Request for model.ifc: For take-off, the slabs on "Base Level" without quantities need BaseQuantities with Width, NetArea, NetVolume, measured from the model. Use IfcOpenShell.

First a look at what the model holds.

```python
import ifcopenshell
import ifcopenshell.util.element
import ifcopenshell.util.unit

model = ifcopenshell.open("model.ifc")
print(model.schema)
for unit_type in ("LENGTHUNIT", "AREAUNIT", "VOLUMEUNIT"):
    print(unit_type, ifcopenshell.util.unit.calculate_unit_scale(model, unit_type))
storey = next(s for s in model.by_type("IfcBuildingStorey") if s.Name == "Base Level")
slabs = [e for e in ifcopenshell.util.element.get_decomposition(storey) if e.is_a("IfcSlab")]
for e in sorted(slabs, key=lambda e: e.id()):
    print(e.id(), e.is_a(), e.Name, list(ifcopenshell.util.element.get_psets(e, qtos_only=True)), sep=" | ")
```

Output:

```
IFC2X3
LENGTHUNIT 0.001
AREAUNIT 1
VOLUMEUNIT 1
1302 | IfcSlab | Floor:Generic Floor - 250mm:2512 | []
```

```python
import ifcopenshell
import ifcopenshell.api.pset
import ifcopenshell.geom
import ifcopenshell.util.element
import ifcopenshell.util.shape
import ifcopenshell.util.unit

model = ifcopenshell.open("model.ifc")
unit_scale = ifcopenshell.util.unit.calculate_unit_scale(model)
area_scale = ifcopenshell.util.unit.calculate_unit_scale(model, "AREAUNIT")
volume_scale = ifcopenshell.util.unit.calculate_unit_scale(model, "VOLUMEUNIT")
settings = ifcopenshell.geom.settings()

storey = next(s for s in model.by_type("IfcBuildingStorey") if s.Name == "Base Level")
slabs = [e for e in ifcopenshell.util.element.get_decomposition(storey) if e.is_a("IfcSlab")]

for e in sorted(slabs, key=lambda e: e.id()):
    if ifcopenshell.util.element.get_psets(e, qtos_only=True, should_inherit=False):
        continue
    # Geometry comes back in metres, in the element's own axes.
    shape = ifcopenshell.geom.create_shape(settings, e)
    values = {
        "Width": ifcopenshell.util.shape.get_z(shape.geometry) / unit_scale,
        "NetArea": ifcopenshell.util.shape.get_footprint_area(shape.geometry) / area_scale,
        "NetVolume": ifcopenshell.util.shape.get_volume(shape.geometry) / volume_scale,
    }
    qto = ifcopenshell.api.pset.add_qto(model, product=e, name="BaseQuantities")
    ifcopenshell.api.pset.edit_qto(model, qto=qto, properties=values)
    print(e.id(), {k: round(v, 3) for k, v in values.items()})

model.write("model-out.ifc")
```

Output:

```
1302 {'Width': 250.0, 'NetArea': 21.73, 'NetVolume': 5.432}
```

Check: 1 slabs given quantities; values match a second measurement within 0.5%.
